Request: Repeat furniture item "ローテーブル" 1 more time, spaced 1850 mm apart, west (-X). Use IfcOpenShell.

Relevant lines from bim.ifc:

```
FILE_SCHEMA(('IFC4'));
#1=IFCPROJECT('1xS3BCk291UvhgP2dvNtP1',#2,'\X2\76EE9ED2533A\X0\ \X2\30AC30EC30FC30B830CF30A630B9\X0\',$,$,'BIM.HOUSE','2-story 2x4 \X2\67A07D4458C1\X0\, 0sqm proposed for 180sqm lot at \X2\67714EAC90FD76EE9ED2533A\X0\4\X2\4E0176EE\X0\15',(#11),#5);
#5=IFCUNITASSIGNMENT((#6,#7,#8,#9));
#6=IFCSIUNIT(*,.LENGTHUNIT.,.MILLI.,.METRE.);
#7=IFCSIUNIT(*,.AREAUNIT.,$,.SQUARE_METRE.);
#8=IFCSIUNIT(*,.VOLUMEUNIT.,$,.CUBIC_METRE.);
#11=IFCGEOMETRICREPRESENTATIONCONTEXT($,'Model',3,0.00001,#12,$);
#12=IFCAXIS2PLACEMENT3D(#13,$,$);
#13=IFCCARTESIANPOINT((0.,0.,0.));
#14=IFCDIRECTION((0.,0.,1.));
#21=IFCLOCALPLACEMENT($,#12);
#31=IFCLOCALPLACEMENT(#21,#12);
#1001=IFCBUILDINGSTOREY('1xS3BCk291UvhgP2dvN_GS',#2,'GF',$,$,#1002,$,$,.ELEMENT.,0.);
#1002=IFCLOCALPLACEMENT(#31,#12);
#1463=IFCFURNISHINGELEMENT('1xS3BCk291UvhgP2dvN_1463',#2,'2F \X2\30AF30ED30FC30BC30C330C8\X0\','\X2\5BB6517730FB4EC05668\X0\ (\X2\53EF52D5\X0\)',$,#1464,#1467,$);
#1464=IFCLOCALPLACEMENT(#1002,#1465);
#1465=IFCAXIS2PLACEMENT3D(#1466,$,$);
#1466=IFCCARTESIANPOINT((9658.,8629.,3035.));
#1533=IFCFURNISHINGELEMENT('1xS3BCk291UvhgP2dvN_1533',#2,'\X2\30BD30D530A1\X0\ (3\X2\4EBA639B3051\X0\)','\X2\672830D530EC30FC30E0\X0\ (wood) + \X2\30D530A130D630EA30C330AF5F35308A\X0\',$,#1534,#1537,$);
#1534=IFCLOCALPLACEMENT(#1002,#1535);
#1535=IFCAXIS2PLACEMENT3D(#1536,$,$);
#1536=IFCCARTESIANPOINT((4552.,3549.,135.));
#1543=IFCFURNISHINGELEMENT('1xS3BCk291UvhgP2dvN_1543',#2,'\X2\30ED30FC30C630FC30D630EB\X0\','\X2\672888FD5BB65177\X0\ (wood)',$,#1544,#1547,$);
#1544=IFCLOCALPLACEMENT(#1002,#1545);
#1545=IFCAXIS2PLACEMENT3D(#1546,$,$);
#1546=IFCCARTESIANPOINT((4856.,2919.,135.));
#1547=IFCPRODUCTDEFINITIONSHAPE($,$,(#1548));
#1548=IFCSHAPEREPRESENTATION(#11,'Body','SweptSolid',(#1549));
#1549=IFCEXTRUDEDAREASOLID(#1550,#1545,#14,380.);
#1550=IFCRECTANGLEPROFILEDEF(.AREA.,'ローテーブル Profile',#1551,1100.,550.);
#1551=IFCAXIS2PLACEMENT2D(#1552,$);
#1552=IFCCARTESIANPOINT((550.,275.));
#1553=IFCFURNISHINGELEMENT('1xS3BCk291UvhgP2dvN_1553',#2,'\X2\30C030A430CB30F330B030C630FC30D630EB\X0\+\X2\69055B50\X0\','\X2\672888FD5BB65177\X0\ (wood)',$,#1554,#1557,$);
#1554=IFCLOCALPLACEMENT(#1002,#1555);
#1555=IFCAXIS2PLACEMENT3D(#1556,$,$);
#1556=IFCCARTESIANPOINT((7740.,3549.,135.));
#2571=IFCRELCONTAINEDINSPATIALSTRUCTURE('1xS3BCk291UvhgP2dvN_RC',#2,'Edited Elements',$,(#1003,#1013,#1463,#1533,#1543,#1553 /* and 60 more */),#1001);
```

```python
import numpy as np
import ifcopenshell
import ifcopenshell.api.geometry
import ifcopenshell.api.root
import ifcopenshell.util.element
import ifcopenshell.util.placement

model = ifcopenshell.open("bim.ifc")


def reuse_history(source, copy):
    """copy_class also copies each property set's owner history, people and application; keep the originals."""
    for rel in copy.IsDefinedBy:
        if rel.is_a("IfcRelDefinesByProperties") and (history := rel.RelatingPropertyDefinition.OwnerHistory):
            rel.RelatingPropertyDefinition.OwnerHistory = source.OwnerHistory
            ifcopenshell.util.element.remove_deep2(model, history)


source = model.by_id(1543)
base = ifcopenshell.util.placement.get_local_placement(source.ObjectPlacement)
step = np.array([-1.0, 0.0, 0.0]) * 1850.0

for i in range(1, 2):
    copy = ifcopenshell.api.root.copy_class(model, product=source)
    copy.Representation = ifcopenshell.util.element.copy_deep(
        model, source.Representation, exclude=["IfcGeometricRepresentationContext", "IfcRepresentationMap"]
    )
    reuse_history(source, copy)
    matrix = base.copy()
    matrix[:3, 3] += i * step
    print("added at", matrix[:3, 3].round(3) + 0.0)
    ifcopenshell.api.geometry.edit_object_placement(model, product=copy, matrix=matrix, is_si=False)

model.write("bim-out.ifc")
```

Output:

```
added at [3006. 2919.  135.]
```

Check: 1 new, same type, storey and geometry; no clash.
